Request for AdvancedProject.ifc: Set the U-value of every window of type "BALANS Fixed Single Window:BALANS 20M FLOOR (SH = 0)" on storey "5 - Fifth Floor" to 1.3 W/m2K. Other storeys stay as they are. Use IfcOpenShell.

First a look at what the model holds.

```python
import ifcopenshell
import ifcopenshell.util.element

model = ifcopenshell.open("AdvancedProject.ifc")
print(model.schema)
storey = next(s for s in model.by_type("IfcBuildingStorey") if s.Name == "5 - Fifth Floor")
windows = [e for e in ifcopenshell.util.element.get_decomposition(storey) if e.is_a("IfcWindow")]
seen = {}
for e in windows:
    element_type = ifcopenshell.util.element.get_type(e)
    key = (element_type.Name if element_type != e and element_type else None, ifcopenshell.util.element.get_pset(e, "Pset_WindowCommon", "ThermalTransmittance"))
    seen[key] = seen.get(key, 0) + 1
for (name, value), count in sorted(seen.items(), key=str):
    print(count, "x", name, "|", value)
```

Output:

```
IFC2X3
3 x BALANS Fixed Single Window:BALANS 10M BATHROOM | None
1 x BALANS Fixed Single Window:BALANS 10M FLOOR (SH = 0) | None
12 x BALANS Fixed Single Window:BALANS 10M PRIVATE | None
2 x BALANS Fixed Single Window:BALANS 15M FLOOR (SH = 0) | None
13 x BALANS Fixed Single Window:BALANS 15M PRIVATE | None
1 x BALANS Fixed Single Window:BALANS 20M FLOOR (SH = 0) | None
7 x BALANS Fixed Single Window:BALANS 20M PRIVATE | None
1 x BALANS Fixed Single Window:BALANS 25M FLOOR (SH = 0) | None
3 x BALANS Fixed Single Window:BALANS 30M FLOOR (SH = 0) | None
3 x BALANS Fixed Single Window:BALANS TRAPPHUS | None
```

```python
import ifcopenshell
import ifcopenshell.api.pset
import ifcopenshell.util.element

model = ifcopenshell.open("AdvancedProject.ifc")

storey = next(s for s in model.by_type("IfcBuildingStorey") if s.Name == "5 - Fifth Floor")
windows = [e for e in ifcopenshell.util.element.get_decomposition(storey) if e.is_a("IfcWindow")]

count = 0
for e in windows:
    element_type = ifcopenshell.util.element.get_type(e)
    if element_type in (None, e) or element_type.Name != "BALANS Fixed Single Window:BALANS 20M FLOOR (SH = 0)":
        continue
    # add_pset returns the element's existing set when there is one.
    pset = ifcopenshell.api.pset.add_pset(model, product=e, name="Pset_WindowCommon")
    ifcopenshell.api.pset.edit_pset(model, pset=pset, properties={"ThermalTransmittance": 1.3})
    count += 1

print(count, "windows updated")

model.write("AdvancedProject_rev.ifc")
```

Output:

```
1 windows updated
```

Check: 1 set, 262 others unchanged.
